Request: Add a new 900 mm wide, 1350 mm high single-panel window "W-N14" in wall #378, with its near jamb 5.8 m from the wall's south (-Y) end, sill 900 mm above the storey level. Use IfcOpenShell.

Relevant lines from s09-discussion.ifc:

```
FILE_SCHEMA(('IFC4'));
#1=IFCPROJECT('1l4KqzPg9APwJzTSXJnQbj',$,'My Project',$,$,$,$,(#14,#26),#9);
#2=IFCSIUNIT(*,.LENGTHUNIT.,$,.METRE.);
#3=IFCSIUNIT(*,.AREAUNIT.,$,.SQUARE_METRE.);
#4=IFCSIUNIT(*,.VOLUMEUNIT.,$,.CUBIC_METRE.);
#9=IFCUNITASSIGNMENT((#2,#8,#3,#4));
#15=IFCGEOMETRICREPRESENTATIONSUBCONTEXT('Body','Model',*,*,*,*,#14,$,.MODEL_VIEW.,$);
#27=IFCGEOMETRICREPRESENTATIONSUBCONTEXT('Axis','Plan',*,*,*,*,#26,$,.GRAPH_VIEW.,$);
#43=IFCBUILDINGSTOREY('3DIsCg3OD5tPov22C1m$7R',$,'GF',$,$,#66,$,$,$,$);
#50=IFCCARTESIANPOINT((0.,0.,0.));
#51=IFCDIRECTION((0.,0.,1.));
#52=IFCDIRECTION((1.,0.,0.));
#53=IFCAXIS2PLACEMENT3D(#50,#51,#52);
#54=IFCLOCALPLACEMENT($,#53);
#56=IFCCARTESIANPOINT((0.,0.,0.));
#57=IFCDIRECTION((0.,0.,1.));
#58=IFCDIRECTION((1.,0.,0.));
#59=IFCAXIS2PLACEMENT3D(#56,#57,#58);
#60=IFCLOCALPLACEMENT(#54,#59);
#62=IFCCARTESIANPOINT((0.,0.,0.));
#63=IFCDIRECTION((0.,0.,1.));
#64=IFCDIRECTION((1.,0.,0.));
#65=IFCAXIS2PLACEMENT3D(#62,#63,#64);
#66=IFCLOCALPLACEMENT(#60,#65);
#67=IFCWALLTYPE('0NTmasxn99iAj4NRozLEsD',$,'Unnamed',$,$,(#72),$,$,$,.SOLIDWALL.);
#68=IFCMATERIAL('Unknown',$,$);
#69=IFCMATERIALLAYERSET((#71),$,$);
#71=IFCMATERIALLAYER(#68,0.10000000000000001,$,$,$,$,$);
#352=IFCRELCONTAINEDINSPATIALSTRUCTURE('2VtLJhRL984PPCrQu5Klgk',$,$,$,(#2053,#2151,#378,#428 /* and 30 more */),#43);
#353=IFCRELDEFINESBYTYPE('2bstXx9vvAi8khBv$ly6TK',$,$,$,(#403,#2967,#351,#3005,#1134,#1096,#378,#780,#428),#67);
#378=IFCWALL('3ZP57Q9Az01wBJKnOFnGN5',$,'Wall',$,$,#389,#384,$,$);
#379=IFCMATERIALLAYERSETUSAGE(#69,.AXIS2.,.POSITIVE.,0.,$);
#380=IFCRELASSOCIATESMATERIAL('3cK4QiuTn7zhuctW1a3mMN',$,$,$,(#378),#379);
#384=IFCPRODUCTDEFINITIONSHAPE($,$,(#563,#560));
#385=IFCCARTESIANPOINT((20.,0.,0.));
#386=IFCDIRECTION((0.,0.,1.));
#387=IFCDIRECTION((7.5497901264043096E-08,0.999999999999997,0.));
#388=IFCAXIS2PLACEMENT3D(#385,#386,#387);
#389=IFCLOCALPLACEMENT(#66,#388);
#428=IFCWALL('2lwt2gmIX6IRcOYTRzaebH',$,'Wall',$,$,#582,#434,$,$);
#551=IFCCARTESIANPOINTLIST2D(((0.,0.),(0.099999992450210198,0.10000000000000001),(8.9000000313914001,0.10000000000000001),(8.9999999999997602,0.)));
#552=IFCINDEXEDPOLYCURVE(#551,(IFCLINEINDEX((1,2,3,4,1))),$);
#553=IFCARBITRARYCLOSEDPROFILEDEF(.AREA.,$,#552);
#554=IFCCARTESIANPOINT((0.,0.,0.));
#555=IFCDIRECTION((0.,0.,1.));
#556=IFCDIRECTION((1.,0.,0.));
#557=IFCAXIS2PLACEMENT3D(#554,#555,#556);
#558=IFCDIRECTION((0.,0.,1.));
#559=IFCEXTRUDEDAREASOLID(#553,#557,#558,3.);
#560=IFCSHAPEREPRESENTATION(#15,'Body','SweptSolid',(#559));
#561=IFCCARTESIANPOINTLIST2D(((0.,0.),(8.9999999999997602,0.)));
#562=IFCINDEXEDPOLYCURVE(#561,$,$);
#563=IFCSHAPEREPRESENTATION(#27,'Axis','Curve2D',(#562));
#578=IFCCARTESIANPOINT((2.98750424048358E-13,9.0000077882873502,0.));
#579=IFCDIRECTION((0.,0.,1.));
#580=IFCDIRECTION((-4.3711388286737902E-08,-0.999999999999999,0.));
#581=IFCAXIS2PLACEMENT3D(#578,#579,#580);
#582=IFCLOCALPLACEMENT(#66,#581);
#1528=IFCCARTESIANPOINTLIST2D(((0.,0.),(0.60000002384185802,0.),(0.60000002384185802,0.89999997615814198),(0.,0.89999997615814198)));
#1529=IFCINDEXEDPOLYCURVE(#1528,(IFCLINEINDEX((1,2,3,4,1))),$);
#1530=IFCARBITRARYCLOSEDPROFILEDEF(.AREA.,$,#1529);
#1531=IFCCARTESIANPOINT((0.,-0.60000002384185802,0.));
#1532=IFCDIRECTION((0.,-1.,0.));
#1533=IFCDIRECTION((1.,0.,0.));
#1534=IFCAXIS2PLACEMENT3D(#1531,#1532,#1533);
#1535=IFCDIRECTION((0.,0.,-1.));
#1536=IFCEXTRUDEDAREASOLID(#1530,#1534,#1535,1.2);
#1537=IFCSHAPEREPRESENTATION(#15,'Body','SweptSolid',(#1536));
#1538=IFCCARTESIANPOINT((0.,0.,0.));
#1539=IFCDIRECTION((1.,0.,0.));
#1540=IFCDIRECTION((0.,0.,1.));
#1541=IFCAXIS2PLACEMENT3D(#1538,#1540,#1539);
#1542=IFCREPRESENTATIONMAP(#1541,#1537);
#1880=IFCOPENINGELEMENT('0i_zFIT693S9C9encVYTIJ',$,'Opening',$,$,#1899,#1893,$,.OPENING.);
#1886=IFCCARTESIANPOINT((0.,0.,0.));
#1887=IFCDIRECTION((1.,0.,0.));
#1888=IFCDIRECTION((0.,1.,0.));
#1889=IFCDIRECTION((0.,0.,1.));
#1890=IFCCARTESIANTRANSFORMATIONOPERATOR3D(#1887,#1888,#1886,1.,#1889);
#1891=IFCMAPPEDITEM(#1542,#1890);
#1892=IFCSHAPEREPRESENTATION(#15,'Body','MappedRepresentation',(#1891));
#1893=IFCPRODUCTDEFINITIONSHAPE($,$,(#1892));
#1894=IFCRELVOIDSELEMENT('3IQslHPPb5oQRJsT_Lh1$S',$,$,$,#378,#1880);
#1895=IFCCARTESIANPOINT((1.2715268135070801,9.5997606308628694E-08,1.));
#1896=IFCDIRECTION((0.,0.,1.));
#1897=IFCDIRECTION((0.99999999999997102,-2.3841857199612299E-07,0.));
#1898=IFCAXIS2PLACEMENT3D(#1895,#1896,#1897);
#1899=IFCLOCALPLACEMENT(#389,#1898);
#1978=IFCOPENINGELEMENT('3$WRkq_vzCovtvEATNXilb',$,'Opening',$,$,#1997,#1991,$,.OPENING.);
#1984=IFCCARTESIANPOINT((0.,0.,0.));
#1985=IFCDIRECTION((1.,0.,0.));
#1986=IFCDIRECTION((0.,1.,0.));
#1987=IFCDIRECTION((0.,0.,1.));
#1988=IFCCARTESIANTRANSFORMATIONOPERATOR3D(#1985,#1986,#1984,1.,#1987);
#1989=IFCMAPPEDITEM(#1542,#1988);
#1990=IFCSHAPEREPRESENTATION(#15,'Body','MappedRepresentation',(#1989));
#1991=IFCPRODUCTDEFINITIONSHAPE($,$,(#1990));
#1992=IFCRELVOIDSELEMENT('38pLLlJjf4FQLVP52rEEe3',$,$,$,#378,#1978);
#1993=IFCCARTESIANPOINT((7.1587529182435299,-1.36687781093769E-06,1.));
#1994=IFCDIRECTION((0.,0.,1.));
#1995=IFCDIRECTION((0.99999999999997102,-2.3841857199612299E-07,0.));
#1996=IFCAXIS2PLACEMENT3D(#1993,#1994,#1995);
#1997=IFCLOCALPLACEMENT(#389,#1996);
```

```python
import numpy as np
import ifcopenshell
import ifcopenshell.api.feature
import ifcopenshell.api.geometry
import ifcopenshell.api.root
import ifcopenshell.api.spatial
import ifcopenshell.geom
import ifcopenshell.util.element
import ifcopenshell.util.placement
import ifcopenshell.util.representation
import ifcopenshell.util.shape
import ifcopenshell.util.unit

model = ifcopenshell.open("s09-discussion.ifc")
unit_scale = ifcopenshell.util.unit.calculate_unit_scale(model)
settings = ifcopenshell.geom.settings()


def volume(element):
    """Net volume in cubic metres, openings subtracted."""
    shape = ifcopenshell.geom.create_shape(settings, element)
    return ifcopenshell.util.shape.get_volume(shape.geometry)


wall = model.by_id(378)
storey = ifcopenshell.util.element.get_container(wall, ifc_class="IfcBuildingStorey")
context = ifcopenshell.util.representation.get_context(model, "Model", "Body", "MODEL_VIEW")
before = volume(wall)

width, height, from_end, sill = 0.9, 1.35, 5.8, 0.9  # metres

# The wall runs along its own X axis, and the end named is its -X end.
wall_shape = ifcopenshell.geom.create_shape(settings, wall)
x, y, z = ifcopenshell.util.shape.get_vertices(wall_shape.geometry).T
start = x.min() + from_end
face, thickness = float(y.min()), float(y.max() - y.min())
wall_matrix = ifcopenshell.util.placement.get_local_placement(wall.ObjectPlacement)
level = ifcopenshell.util.placement.get_local_placement(storey.ObjectPlacement)[2, 3]


def in_wall(x, y):
    """Placement at x, y metres in the wall's axes, at sill height."""
    matrix = wall_matrix.copy()
    matrix[:, 3] = wall_matrix @ np.array([x / unit_scale, y / unit_scale, 0.0, 1.0])
    matrix[2, 3] = level + sill / unit_scale
    return matrix


# Opening: a box that overshoots both wall faces by 50 mm.
opening = ifcopenshell.api.root.create_entity(model, ifc_class="IfcOpeningElement", predefined_type="OPENING")
box = ifcopenshell.api.geometry.add_wall_representation(
    model, context=context, length=width, height=height, thickness=thickness + 0.1
)
ifcopenshell.api.geometry.assign_representation(model, product=opening, representation=box)
ifcopenshell.api.geometry.edit_object_placement(model, product=opening, matrix=in_wall(start, face - 0.05), is_si=False)
ifcopenshell.api.feature.add_feature(model, feature=opening, element=wall)

window = ifcopenshell.api.root.create_entity(model, ifc_class="IfcWindow", name="W-N14", predefined_type="WINDOW")
window.OverallWidth, window.OverallHeight = width / unit_scale, height / unit_scale
window.PartitioningType = "SINGLE_PANEL"
body = ifcopenshell.api.geometry.add_window_representation(
    model,
    context=context,
    overall_width=window.OverallWidth,
    overall_height=window.OverallHeight,
    partition_type="SINGLE_PANEL",
)
ifcopenshell.api.geometry.assign_representation(model, product=window, representation=body)
ifcopenshell.api.spatial.assign_container(model, products=[window], relating_structure=storey)
ifcopenshell.api.feature.add_filling(model, opening=opening, element=window)

# Centre the window in the wall's thickness.
ifcopenshell.api.geometry.edit_object_placement(model, product=window, matrix=in_wall(start, face), is_si=False)
window_shape = ifcopenshell.geom.create_shape(settings, window)
depth = ifcopenshell.util.shape.get_vertices(window_shape.geometry)[:, 1]
offset = face + thickness / 2 - (depth.min() + depth.max()) / 2
ifcopenshell.api.geometry.edit_object_placement(model, product=window, matrix=in_wall(start, offset), is_si=False)

after = volume(wall)

print(f"wall volume {before:.3f} -> {after:.3f} m3")

model.write("s09-discussion_edited.ifc")
```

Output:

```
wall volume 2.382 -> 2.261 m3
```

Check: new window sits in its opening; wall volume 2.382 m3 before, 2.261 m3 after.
